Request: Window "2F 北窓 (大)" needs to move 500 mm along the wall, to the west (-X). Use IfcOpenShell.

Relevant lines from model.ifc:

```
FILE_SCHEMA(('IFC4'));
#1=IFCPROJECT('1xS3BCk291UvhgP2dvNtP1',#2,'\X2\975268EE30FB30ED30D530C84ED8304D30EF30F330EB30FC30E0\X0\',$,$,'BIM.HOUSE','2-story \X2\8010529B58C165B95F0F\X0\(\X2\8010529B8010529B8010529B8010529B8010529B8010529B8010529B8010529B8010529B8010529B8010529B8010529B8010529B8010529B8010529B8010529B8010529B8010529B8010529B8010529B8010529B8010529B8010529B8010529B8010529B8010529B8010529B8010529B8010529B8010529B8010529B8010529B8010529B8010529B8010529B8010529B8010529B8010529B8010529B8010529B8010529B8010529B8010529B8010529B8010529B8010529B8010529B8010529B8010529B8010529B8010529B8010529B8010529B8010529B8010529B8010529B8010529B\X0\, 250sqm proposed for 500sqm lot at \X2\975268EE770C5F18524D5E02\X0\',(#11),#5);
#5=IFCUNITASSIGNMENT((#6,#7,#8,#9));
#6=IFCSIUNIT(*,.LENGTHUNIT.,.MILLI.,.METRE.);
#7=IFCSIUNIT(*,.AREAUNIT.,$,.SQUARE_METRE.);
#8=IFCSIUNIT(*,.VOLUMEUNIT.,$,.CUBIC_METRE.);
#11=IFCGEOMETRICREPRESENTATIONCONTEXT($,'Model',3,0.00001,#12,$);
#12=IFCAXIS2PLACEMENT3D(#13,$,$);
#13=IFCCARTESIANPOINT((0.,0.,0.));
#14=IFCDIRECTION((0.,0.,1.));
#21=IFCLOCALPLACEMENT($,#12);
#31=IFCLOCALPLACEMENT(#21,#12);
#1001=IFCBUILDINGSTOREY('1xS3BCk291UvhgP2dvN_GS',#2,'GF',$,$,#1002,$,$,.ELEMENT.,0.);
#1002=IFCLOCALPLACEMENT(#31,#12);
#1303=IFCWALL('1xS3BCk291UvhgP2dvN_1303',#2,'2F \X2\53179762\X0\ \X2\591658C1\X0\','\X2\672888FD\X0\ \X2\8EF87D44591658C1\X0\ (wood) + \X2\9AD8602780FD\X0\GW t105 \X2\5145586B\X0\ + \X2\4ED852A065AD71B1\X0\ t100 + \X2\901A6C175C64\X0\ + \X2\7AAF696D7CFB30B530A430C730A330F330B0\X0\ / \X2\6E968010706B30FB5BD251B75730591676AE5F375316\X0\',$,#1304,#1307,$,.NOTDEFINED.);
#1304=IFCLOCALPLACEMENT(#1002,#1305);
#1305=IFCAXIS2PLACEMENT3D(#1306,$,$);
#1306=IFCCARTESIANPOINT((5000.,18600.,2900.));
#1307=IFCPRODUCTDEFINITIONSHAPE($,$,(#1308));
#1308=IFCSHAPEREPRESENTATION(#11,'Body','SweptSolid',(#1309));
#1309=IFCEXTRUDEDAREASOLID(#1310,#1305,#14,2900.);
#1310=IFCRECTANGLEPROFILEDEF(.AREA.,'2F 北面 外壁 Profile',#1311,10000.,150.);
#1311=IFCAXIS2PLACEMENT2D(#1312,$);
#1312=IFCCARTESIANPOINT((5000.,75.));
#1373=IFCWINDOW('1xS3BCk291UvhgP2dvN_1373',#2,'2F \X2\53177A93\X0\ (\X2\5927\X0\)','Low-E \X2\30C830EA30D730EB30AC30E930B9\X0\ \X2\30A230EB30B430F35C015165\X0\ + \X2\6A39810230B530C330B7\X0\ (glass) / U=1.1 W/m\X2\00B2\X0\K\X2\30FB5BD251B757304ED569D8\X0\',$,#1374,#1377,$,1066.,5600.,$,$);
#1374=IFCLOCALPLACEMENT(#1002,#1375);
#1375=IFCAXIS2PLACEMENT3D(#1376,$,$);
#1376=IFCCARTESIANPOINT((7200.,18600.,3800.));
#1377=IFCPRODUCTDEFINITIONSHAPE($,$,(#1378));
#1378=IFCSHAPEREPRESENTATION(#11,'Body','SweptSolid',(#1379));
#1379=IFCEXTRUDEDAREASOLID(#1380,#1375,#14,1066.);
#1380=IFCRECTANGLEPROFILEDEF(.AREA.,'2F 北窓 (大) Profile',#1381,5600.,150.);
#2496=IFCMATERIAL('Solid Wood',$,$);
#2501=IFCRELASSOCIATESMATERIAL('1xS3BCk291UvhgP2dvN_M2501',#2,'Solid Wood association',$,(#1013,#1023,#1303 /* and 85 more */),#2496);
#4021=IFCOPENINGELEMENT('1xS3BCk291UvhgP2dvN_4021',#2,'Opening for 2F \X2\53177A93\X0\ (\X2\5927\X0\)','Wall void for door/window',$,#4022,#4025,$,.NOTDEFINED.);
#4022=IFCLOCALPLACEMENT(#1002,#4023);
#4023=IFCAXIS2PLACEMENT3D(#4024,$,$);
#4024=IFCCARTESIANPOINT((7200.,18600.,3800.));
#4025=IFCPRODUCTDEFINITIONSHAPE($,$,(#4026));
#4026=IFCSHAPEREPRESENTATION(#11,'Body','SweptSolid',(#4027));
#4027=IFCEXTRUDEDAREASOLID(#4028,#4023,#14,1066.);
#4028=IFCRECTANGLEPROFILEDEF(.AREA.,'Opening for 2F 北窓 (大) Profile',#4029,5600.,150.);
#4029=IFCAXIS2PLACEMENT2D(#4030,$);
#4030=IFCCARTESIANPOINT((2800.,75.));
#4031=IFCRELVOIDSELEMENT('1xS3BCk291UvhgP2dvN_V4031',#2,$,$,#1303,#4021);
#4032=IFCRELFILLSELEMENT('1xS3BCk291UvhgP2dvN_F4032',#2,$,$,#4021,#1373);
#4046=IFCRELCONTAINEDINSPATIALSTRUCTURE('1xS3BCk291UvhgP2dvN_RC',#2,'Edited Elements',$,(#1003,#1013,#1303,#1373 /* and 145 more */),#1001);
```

```python
import ifcopenshell
import ifcopenshell.api.geometry
import ifcopenshell.util.placement

model = ifcopenshell.open("model.ifc")

window = model.by_guid("1xS3BCk291UvhgP2dvN_1373")
opening = window.FillsVoids[0].RelatingOpeningElement
wall = opening.VoidsElements[0].RelatingBuildingElement

wall_matrix = ifcopenshell.util.placement.get_local_placement(wall.ObjectPlacement)
shift = wall_matrix[:3, 0] * -500.0
before = ifcopenshell.util.placement.get_local_placement(window.ObjectPlacement)[:3, 3].copy()

# The window is not placed relative to its opening, so move both.
for product in (opening, window):
    matrix = ifcopenshell.util.placement.get_local_placement(product.ObjectPlacement)
    matrix[:3, 3] += shift
    ifcopenshell.api.geometry.edit_object_placement(model, product=product, matrix=matrix, is_si=False)

after = ifcopenshell.util.placement.get_local_placement(window.ObjectPlacement)[:3, 3]
print("window moved by", (after - before).round(3) + 0.0)

model.write("model_v2.ifc")
```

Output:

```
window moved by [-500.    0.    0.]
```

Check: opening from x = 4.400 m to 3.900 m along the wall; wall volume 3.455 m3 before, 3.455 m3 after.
